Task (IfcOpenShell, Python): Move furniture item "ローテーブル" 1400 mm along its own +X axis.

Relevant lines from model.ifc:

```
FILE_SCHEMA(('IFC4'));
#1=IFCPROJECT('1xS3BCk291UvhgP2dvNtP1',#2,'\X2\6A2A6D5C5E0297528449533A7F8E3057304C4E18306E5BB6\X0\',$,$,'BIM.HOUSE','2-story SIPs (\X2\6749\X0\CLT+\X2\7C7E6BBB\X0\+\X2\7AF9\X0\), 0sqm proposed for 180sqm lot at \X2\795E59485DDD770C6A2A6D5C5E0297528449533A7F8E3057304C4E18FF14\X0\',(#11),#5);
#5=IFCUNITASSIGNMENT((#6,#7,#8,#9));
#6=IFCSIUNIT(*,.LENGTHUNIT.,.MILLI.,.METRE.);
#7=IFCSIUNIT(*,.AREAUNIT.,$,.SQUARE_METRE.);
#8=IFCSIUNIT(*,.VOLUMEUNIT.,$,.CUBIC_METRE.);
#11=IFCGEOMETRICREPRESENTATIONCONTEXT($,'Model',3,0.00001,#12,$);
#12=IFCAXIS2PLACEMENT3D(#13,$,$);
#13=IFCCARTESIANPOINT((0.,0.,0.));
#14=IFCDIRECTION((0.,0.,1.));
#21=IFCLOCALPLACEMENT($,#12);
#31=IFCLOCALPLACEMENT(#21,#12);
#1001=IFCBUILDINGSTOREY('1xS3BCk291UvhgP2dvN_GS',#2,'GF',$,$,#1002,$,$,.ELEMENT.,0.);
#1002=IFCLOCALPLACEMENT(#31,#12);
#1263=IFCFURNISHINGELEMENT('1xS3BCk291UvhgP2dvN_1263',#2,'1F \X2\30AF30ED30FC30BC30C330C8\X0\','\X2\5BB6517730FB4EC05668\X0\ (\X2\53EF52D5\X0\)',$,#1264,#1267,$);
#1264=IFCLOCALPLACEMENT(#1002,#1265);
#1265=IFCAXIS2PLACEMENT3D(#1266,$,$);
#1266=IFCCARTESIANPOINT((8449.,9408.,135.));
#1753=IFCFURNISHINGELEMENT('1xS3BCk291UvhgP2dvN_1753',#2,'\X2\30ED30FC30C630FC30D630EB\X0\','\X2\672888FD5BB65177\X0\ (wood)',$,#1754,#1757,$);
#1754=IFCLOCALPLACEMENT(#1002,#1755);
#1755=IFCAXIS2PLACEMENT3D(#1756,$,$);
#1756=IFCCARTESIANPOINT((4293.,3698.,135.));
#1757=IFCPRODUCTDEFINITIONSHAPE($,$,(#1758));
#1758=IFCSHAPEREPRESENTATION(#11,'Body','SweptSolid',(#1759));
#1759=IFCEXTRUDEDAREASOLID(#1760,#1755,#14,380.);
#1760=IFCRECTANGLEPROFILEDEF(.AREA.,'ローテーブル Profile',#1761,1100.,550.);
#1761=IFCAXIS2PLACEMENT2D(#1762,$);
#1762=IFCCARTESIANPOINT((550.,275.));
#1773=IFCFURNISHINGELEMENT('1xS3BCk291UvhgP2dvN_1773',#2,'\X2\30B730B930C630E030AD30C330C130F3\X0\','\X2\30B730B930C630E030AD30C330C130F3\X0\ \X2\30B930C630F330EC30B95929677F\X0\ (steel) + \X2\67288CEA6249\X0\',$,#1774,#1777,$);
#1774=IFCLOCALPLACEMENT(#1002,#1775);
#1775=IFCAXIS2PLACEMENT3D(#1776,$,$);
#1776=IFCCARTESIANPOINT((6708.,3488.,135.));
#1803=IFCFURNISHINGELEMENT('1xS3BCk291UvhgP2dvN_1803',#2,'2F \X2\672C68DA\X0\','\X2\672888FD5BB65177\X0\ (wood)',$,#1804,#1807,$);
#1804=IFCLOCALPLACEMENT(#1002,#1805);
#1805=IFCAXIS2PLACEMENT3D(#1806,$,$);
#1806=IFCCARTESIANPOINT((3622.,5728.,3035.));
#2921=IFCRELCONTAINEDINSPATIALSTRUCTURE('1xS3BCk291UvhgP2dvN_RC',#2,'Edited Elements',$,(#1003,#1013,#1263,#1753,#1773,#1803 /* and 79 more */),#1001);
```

```python
import ifcopenshell
import ifcopenshell.api.geometry
import ifcopenshell.util.placement

model = ifcopenshell.open("model.ifc")

item = model.by_guid("1xS3BCk291UvhgP2dvN_1753")
matrix = ifcopenshell.util.placement.get_local_placement(item.ObjectPlacement)
matrix[:3, 3] += matrix[:3, 0] * 1400.0
ifcopenshell.api.geometry.edit_object_placement(model, product=item, matrix=matrix, is_si=False)

print(ifcopenshell.util.placement.get_local_placement(item.ObjectPlacement).round(3) + 0.0)

model.write("model_rev.ifc")
```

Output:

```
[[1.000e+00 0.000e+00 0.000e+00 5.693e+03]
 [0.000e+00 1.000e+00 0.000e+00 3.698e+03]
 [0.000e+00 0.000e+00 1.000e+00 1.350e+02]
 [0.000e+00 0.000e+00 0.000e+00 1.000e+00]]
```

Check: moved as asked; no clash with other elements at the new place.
